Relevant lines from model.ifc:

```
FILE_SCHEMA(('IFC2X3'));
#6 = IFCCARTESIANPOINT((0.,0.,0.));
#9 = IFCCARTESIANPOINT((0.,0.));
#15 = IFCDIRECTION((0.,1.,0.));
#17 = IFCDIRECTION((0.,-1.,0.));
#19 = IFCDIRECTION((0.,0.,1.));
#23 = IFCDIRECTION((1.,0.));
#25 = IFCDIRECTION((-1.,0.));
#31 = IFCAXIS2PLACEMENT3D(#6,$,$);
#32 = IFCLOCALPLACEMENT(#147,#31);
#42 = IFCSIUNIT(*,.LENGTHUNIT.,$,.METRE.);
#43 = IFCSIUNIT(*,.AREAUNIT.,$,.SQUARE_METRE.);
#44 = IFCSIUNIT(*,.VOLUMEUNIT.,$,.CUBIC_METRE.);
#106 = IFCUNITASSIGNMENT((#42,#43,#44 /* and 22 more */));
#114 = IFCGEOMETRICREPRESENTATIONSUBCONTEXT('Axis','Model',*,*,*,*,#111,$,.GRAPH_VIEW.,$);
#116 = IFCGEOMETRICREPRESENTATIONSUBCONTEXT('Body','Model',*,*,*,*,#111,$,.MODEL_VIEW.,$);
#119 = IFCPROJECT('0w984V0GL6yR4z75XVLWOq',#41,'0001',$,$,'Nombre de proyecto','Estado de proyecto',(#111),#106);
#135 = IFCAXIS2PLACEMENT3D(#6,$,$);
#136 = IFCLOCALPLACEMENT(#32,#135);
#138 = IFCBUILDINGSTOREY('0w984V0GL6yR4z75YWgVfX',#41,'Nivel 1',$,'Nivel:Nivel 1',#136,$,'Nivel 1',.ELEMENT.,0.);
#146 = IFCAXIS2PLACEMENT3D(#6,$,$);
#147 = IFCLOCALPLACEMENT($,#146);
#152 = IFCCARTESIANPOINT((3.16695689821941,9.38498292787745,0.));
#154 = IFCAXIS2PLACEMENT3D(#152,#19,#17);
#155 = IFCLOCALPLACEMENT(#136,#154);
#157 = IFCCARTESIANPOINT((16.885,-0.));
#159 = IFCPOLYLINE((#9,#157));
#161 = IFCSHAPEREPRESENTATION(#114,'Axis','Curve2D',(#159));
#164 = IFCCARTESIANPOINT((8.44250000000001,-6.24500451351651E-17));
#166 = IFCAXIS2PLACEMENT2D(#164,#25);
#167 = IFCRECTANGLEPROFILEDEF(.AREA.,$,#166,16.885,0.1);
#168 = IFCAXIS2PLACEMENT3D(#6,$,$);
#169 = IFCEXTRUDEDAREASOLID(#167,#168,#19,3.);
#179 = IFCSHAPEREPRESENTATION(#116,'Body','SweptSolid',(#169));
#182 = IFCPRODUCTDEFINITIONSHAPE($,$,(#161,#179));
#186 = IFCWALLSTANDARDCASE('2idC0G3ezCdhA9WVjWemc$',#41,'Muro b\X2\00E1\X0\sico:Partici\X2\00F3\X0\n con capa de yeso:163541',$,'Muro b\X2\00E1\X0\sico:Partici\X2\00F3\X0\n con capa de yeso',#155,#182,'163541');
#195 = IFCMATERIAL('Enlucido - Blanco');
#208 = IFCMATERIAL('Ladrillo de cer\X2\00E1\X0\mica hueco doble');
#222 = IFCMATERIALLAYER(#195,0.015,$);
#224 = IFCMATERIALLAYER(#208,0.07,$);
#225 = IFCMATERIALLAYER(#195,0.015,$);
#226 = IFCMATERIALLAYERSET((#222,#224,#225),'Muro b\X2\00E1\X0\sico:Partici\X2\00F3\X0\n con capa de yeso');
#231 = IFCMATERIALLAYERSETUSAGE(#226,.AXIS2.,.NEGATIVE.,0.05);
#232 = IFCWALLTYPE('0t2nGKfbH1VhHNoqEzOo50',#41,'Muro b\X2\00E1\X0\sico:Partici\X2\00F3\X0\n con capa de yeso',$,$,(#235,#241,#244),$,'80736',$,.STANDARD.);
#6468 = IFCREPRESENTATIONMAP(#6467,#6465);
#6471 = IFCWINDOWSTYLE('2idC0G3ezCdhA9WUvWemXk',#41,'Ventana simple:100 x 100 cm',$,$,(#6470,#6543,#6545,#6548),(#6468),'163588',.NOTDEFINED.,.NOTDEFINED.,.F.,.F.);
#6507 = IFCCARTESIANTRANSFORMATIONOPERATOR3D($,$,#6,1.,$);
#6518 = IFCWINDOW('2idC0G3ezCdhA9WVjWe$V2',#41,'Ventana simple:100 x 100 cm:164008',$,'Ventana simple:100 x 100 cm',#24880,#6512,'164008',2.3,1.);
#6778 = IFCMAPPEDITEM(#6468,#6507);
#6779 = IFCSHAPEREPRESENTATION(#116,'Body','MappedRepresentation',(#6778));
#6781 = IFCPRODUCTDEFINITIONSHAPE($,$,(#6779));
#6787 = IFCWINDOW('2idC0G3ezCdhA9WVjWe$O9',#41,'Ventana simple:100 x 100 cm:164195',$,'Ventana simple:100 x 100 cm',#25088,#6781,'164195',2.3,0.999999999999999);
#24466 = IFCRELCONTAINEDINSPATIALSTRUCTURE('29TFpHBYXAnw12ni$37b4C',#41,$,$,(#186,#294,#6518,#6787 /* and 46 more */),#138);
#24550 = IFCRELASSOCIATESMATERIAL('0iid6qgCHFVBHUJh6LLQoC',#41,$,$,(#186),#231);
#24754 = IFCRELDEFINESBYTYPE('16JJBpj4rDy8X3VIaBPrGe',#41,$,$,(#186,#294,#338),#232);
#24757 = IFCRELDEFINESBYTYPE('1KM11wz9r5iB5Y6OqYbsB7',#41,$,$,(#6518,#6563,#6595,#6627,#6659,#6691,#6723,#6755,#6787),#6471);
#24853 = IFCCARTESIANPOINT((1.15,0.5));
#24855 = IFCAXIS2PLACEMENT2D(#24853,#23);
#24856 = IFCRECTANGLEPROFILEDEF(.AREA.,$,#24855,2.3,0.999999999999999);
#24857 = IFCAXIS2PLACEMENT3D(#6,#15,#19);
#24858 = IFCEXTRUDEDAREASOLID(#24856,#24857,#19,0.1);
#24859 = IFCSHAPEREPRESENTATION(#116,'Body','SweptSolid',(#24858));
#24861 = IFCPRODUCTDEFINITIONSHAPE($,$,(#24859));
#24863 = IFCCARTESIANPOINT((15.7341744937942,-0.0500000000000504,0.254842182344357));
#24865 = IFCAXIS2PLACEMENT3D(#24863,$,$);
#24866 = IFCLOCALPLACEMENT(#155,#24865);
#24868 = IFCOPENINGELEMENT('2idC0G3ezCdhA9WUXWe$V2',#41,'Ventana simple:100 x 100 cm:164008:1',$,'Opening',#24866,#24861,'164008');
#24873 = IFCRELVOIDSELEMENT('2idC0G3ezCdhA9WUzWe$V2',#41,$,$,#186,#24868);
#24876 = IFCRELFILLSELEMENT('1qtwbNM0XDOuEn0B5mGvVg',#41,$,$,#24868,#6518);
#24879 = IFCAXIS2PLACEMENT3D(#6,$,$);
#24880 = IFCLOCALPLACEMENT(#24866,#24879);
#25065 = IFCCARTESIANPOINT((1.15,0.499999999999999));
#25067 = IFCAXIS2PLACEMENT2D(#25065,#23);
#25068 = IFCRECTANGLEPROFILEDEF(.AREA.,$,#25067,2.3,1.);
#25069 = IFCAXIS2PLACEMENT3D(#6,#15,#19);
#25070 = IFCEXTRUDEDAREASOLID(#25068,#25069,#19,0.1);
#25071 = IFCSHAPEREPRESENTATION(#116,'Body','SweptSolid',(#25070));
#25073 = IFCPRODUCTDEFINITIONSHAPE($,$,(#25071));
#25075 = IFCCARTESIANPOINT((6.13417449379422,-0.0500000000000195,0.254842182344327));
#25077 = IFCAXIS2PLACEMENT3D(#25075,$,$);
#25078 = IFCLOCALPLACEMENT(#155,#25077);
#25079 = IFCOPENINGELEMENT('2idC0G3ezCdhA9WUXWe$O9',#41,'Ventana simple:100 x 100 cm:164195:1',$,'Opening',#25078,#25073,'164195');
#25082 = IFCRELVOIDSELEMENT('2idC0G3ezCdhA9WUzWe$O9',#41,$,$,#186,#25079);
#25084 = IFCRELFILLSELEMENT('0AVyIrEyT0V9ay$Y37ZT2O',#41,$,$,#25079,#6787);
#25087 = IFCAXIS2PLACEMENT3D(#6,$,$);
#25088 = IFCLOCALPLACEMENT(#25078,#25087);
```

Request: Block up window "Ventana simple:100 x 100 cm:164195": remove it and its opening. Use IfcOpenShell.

```python
import ifcopenshell
import ifcopenshell.api.feature
import ifcopenshell.api.root
import ifcopenshell.geom
import ifcopenshell.util.shape

model = ifcopenshell.open("model.ifc")
settings = ifcopenshell.geom.settings()


def volume(element):
    """Net volume in cubic metres, openings subtracted."""
    shape = ifcopenshell.geom.create_shape(settings, element)
    return ifcopenshell.util.shape.get_volume(shape.geometry)


window = model.by_guid("2idC0G3ezCdhA9WVjWe$O9")
opening = window.FillsVoids[0].RelatingOpeningElement
wall = opening.VoidsElements[0].RelatingBuildingElement
before = volume(wall)

ifcopenshell.api.root.remove_product(model, product=window)
ifcopenshell.api.feature.remove_feature(model, feature=opening)

after = volume(wall)

print(f"wall volume {before:.3f} -> {after:.3f} m3")

model.write("model-out.ifc")
```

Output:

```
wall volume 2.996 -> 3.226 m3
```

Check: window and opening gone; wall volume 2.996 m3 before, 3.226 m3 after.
